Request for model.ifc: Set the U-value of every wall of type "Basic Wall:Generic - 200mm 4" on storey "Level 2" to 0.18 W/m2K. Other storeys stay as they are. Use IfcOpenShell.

First a look at what the model holds.

```python
import ifcopenshell
import ifcopenshell.util.element

model = ifcopenshell.open("model.ifc")
print(model.schema)
storey = next(s for s in model.by_type("IfcBuildingStorey") if s.Name == "Level 2")
walls = [e for e in ifcopenshell.util.element.get_decomposition(storey) if e.is_a("IfcWall")]
seen = {}
for e in walls:
    element_type = ifcopenshell.util.element.get_type(e)
    key = (element_type.Name if element_type != e and element_type else None, ifcopenshell.util.element.get_pset(e, "Pset_WallCommon", "ThermalTransmittance"))
    seen[key] = seen.get(key, 0) + 1
for (name, value), count in sorted(seen.items(), key=str):
    print(count, "x", name, "|", value)
```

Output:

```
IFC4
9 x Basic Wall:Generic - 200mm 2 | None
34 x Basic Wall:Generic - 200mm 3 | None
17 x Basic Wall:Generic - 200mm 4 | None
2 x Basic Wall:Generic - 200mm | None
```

```python
import ifcopenshell
import ifcopenshell.api.pset
import ifcopenshell.util.element

model = ifcopenshell.open("model.ifc")

storey = next(s for s in model.by_type("IfcBuildingStorey") if s.Name == "Level 2")
walls = [e for e in ifcopenshell.util.element.get_decomposition(storey) if e.is_a("IfcWall")]

count = 0
for e in walls:
    element_type = ifcopenshell.util.element.get_type(e)
    if element_type in (None, e) or element_type.Name != "Basic Wall:Generic - 200mm 4":
        continue
    # add_pset returns the element's existing set when there is one.
    pset = ifcopenshell.api.pset.add_pset(model, product=e, name="Pset_WallCommon")
    ifcopenshell.api.pset.edit_pset(model, pset=pset, properties={"ThermalTransmittance": 0.18})
    count += 1

print(count, "walls updated")

model.write("model_edited.ifc")
```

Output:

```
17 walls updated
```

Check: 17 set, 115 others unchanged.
